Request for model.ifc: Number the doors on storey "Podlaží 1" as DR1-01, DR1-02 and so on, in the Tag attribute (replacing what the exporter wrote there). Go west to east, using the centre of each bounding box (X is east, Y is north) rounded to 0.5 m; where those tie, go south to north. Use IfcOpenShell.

First a look at what the model holds.

```python
import ifcopenshell
import ifcopenshell.util.element
import ifcopenshell.util.placement

model = ifcopenshell.open("model.ifc")
print(model.schema)
storey = next(s for s in model.by_type("IfcBuildingStorey") if s.Name == "Podlaží 1")
doors = [e for e in ifcopenshell.util.element.get_decomposition(storey) if e.is_a("IfcDoor")]
for e in sorted(doors, key=lambda e: e.id()):
    origin = ifcopenshell.util.placement.get_local_placement(e.ObjectPlacement)[:3, 3]
    print(e.id(), e.Tag, e.Name, origin.round(2) + 0.0, sep=" | ")
```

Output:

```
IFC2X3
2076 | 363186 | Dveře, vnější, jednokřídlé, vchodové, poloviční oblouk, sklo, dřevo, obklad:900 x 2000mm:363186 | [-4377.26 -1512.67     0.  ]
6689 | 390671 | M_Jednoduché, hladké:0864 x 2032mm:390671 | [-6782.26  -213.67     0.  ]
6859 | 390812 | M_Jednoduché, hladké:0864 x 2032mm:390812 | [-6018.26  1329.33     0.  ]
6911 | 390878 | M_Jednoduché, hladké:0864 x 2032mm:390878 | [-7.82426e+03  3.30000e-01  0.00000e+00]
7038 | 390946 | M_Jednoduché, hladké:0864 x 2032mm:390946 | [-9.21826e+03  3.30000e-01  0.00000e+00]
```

```python
import ifcopenshell
import ifcopenshell.geom
import ifcopenshell.util.element
import ifcopenshell.util.shape

model = ifcopenshell.open("model.ifc")
settings = ifcopenshell.geom.settings()
settings.set("use-world-coords", True)


def centre(element):
    shape = ifcopenshell.geom.create_shape(settings, element)
    return ifcopenshell.util.shape.get_bbox_centroid(shape.geometry)


storey = next(s for s in model.by_type("IfcBuildingStorey") if s.Name == "Podlaží 1")
doors = [e for e in ifcopenshell.util.element.get_decomposition(storey) if e.is_a("IfcDoor")]

# Insertion points can sit at a corner or the storey origin, so sort by the geometry (in metres).
centres = {e: centre(e) for e in doors}
doors.sort(key=lambda e: (round(centres[e][0] / 0.5), centres[e][1]))

for i, e in enumerate(doors, start=1):
    number = f"DR1-{i:02d}"
    e.Tag = number
    print(e.id(), number)

model.write("model_v2.ifc")
```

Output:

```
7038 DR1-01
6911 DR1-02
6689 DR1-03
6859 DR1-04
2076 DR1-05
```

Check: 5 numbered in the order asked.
